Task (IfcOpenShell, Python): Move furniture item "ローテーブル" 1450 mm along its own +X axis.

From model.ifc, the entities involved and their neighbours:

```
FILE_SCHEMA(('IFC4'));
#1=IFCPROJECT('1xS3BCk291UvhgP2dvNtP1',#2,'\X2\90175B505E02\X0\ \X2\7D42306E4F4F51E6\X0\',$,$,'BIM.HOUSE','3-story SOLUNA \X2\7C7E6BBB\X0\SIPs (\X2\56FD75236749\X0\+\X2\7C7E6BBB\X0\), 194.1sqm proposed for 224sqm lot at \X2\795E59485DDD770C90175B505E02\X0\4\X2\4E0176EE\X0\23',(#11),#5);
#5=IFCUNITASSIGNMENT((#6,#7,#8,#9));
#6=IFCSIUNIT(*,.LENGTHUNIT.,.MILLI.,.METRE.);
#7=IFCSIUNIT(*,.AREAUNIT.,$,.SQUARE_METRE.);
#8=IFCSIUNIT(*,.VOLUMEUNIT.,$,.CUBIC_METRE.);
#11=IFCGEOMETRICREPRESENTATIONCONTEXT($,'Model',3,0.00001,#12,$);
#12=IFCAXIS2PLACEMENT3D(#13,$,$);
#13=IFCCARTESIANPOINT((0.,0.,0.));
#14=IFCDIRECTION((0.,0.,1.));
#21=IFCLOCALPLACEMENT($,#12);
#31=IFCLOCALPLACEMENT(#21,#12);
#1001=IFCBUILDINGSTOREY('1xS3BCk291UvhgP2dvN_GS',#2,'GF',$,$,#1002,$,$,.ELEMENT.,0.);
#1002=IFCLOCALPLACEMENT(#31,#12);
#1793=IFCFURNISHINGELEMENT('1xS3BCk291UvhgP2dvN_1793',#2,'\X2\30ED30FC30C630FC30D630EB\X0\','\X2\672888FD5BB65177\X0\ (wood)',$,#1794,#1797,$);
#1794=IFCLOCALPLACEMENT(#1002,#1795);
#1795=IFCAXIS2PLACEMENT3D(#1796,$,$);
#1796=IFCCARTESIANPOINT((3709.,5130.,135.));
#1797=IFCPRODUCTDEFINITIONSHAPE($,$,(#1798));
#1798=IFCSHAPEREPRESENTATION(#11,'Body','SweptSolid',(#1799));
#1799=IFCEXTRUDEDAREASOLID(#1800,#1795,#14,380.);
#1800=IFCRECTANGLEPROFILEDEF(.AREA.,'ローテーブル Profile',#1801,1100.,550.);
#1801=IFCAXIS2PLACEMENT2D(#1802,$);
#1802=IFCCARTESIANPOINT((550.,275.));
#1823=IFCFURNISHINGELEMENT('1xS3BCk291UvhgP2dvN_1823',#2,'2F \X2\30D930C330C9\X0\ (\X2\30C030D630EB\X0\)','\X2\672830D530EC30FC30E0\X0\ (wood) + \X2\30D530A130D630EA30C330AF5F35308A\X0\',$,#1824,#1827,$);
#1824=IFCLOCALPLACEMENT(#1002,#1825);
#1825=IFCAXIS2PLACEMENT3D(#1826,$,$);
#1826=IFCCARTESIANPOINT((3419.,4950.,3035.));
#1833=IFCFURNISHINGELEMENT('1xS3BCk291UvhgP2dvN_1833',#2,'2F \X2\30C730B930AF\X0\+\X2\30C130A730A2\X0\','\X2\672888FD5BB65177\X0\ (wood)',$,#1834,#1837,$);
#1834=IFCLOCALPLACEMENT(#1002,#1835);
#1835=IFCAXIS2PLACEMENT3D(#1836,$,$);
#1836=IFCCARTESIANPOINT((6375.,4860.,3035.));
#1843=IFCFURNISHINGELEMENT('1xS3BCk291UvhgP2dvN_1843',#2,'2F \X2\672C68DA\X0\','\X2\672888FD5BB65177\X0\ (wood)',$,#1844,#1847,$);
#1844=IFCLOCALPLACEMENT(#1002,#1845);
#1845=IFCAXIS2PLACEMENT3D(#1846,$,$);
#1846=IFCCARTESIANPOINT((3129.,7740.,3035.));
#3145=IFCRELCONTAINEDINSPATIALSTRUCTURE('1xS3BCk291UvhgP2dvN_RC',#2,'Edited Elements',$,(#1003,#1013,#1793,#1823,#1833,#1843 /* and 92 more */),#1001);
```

```python
import ifcopenshell
import ifcopenshell.api.geometry
import ifcopenshell.util.placement

model = ifcopenshell.open("model.ifc")

item = model.by_guid("1xS3BCk291UvhgP2dvN_1793")
matrix = ifcopenshell.util.placement.get_local_placement(item.ObjectPlacement)
matrix[:3, 3] += matrix[:3, 0] * 1450.0
ifcopenshell.api.geometry.edit_object_placement(model, product=item, matrix=matrix, is_si=False)

print(ifcopenshell.util.placement.get_local_placement(item.ObjectPlacement).round(3) + 0.0)

model.write("model_v2.ifc")
```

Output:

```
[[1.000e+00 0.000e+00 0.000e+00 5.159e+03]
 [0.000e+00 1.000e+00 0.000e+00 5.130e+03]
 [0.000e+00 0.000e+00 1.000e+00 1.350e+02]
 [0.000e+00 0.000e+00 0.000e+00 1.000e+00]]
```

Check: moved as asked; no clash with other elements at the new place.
